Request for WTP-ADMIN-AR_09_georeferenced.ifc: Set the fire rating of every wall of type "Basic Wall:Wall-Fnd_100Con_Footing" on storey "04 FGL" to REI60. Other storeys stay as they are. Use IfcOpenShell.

First a look at what the model holds.

```python
import ifcopenshell
import ifcopenshell.util.element

model = ifcopenshell.open("WTP-ADMIN-AR_09_georeferenced.ifc")
print(model.schema)
storey = next(s for s in model.by_type("IfcBuildingStorey") if s.Name == "04 FGL")
walls = [e for e in ifcopenshell.util.element.get_decomposition(storey) if e.is_a("IfcWall")]
seen = {}
for e in walls:
    element_type = ifcopenshell.util.element.get_type(e)
    key = (element_type.Name if element_type != e and element_type else None, ifcopenshell.util.element.get_pset(e, "Pset_WallCommon", "FireRating"))
    seen[key] = seen.get(key, 0) + 1
for (name, value), count in sorted(seen.items(), key=str):
    print(count, "x", name, "|", value)
```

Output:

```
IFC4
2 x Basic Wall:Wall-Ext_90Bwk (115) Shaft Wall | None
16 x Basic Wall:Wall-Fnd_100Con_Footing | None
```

```python
import ifcopenshell
import ifcopenshell.api.pset
import ifcopenshell.util.element

model = ifcopenshell.open("WTP-ADMIN-AR_09_georeferenced.ifc")

storey = next(s for s in model.by_type("IfcBuildingStorey") if s.Name == "04 FGL")
walls = [e for e in ifcopenshell.util.element.get_decomposition(storey) if e.is_a("IfcWall")]

count = 0
for e in walls:
    element_type = ifcopenshell.util.element.get_type(e)
    if element_type in (None, e) or element_type.Name != "Basic Wall:Wall-Fnd_100Con_Footing":
        continue
    # add_pset returns the element's existing set when there is one.
    pset = ifcopenshell.api.pset.add_pset(model, product=e, name="Pset_WallCommon")
    ifcopenshell.api.pset.edit_pset(model, pset=pset, properties={"FireRating": "REI60"})
    count += 1

print(count, "walls updated")

model.write("WTP-ADMIN-AR_09_georeferenced-out.ifc")
```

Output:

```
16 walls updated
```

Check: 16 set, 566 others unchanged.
